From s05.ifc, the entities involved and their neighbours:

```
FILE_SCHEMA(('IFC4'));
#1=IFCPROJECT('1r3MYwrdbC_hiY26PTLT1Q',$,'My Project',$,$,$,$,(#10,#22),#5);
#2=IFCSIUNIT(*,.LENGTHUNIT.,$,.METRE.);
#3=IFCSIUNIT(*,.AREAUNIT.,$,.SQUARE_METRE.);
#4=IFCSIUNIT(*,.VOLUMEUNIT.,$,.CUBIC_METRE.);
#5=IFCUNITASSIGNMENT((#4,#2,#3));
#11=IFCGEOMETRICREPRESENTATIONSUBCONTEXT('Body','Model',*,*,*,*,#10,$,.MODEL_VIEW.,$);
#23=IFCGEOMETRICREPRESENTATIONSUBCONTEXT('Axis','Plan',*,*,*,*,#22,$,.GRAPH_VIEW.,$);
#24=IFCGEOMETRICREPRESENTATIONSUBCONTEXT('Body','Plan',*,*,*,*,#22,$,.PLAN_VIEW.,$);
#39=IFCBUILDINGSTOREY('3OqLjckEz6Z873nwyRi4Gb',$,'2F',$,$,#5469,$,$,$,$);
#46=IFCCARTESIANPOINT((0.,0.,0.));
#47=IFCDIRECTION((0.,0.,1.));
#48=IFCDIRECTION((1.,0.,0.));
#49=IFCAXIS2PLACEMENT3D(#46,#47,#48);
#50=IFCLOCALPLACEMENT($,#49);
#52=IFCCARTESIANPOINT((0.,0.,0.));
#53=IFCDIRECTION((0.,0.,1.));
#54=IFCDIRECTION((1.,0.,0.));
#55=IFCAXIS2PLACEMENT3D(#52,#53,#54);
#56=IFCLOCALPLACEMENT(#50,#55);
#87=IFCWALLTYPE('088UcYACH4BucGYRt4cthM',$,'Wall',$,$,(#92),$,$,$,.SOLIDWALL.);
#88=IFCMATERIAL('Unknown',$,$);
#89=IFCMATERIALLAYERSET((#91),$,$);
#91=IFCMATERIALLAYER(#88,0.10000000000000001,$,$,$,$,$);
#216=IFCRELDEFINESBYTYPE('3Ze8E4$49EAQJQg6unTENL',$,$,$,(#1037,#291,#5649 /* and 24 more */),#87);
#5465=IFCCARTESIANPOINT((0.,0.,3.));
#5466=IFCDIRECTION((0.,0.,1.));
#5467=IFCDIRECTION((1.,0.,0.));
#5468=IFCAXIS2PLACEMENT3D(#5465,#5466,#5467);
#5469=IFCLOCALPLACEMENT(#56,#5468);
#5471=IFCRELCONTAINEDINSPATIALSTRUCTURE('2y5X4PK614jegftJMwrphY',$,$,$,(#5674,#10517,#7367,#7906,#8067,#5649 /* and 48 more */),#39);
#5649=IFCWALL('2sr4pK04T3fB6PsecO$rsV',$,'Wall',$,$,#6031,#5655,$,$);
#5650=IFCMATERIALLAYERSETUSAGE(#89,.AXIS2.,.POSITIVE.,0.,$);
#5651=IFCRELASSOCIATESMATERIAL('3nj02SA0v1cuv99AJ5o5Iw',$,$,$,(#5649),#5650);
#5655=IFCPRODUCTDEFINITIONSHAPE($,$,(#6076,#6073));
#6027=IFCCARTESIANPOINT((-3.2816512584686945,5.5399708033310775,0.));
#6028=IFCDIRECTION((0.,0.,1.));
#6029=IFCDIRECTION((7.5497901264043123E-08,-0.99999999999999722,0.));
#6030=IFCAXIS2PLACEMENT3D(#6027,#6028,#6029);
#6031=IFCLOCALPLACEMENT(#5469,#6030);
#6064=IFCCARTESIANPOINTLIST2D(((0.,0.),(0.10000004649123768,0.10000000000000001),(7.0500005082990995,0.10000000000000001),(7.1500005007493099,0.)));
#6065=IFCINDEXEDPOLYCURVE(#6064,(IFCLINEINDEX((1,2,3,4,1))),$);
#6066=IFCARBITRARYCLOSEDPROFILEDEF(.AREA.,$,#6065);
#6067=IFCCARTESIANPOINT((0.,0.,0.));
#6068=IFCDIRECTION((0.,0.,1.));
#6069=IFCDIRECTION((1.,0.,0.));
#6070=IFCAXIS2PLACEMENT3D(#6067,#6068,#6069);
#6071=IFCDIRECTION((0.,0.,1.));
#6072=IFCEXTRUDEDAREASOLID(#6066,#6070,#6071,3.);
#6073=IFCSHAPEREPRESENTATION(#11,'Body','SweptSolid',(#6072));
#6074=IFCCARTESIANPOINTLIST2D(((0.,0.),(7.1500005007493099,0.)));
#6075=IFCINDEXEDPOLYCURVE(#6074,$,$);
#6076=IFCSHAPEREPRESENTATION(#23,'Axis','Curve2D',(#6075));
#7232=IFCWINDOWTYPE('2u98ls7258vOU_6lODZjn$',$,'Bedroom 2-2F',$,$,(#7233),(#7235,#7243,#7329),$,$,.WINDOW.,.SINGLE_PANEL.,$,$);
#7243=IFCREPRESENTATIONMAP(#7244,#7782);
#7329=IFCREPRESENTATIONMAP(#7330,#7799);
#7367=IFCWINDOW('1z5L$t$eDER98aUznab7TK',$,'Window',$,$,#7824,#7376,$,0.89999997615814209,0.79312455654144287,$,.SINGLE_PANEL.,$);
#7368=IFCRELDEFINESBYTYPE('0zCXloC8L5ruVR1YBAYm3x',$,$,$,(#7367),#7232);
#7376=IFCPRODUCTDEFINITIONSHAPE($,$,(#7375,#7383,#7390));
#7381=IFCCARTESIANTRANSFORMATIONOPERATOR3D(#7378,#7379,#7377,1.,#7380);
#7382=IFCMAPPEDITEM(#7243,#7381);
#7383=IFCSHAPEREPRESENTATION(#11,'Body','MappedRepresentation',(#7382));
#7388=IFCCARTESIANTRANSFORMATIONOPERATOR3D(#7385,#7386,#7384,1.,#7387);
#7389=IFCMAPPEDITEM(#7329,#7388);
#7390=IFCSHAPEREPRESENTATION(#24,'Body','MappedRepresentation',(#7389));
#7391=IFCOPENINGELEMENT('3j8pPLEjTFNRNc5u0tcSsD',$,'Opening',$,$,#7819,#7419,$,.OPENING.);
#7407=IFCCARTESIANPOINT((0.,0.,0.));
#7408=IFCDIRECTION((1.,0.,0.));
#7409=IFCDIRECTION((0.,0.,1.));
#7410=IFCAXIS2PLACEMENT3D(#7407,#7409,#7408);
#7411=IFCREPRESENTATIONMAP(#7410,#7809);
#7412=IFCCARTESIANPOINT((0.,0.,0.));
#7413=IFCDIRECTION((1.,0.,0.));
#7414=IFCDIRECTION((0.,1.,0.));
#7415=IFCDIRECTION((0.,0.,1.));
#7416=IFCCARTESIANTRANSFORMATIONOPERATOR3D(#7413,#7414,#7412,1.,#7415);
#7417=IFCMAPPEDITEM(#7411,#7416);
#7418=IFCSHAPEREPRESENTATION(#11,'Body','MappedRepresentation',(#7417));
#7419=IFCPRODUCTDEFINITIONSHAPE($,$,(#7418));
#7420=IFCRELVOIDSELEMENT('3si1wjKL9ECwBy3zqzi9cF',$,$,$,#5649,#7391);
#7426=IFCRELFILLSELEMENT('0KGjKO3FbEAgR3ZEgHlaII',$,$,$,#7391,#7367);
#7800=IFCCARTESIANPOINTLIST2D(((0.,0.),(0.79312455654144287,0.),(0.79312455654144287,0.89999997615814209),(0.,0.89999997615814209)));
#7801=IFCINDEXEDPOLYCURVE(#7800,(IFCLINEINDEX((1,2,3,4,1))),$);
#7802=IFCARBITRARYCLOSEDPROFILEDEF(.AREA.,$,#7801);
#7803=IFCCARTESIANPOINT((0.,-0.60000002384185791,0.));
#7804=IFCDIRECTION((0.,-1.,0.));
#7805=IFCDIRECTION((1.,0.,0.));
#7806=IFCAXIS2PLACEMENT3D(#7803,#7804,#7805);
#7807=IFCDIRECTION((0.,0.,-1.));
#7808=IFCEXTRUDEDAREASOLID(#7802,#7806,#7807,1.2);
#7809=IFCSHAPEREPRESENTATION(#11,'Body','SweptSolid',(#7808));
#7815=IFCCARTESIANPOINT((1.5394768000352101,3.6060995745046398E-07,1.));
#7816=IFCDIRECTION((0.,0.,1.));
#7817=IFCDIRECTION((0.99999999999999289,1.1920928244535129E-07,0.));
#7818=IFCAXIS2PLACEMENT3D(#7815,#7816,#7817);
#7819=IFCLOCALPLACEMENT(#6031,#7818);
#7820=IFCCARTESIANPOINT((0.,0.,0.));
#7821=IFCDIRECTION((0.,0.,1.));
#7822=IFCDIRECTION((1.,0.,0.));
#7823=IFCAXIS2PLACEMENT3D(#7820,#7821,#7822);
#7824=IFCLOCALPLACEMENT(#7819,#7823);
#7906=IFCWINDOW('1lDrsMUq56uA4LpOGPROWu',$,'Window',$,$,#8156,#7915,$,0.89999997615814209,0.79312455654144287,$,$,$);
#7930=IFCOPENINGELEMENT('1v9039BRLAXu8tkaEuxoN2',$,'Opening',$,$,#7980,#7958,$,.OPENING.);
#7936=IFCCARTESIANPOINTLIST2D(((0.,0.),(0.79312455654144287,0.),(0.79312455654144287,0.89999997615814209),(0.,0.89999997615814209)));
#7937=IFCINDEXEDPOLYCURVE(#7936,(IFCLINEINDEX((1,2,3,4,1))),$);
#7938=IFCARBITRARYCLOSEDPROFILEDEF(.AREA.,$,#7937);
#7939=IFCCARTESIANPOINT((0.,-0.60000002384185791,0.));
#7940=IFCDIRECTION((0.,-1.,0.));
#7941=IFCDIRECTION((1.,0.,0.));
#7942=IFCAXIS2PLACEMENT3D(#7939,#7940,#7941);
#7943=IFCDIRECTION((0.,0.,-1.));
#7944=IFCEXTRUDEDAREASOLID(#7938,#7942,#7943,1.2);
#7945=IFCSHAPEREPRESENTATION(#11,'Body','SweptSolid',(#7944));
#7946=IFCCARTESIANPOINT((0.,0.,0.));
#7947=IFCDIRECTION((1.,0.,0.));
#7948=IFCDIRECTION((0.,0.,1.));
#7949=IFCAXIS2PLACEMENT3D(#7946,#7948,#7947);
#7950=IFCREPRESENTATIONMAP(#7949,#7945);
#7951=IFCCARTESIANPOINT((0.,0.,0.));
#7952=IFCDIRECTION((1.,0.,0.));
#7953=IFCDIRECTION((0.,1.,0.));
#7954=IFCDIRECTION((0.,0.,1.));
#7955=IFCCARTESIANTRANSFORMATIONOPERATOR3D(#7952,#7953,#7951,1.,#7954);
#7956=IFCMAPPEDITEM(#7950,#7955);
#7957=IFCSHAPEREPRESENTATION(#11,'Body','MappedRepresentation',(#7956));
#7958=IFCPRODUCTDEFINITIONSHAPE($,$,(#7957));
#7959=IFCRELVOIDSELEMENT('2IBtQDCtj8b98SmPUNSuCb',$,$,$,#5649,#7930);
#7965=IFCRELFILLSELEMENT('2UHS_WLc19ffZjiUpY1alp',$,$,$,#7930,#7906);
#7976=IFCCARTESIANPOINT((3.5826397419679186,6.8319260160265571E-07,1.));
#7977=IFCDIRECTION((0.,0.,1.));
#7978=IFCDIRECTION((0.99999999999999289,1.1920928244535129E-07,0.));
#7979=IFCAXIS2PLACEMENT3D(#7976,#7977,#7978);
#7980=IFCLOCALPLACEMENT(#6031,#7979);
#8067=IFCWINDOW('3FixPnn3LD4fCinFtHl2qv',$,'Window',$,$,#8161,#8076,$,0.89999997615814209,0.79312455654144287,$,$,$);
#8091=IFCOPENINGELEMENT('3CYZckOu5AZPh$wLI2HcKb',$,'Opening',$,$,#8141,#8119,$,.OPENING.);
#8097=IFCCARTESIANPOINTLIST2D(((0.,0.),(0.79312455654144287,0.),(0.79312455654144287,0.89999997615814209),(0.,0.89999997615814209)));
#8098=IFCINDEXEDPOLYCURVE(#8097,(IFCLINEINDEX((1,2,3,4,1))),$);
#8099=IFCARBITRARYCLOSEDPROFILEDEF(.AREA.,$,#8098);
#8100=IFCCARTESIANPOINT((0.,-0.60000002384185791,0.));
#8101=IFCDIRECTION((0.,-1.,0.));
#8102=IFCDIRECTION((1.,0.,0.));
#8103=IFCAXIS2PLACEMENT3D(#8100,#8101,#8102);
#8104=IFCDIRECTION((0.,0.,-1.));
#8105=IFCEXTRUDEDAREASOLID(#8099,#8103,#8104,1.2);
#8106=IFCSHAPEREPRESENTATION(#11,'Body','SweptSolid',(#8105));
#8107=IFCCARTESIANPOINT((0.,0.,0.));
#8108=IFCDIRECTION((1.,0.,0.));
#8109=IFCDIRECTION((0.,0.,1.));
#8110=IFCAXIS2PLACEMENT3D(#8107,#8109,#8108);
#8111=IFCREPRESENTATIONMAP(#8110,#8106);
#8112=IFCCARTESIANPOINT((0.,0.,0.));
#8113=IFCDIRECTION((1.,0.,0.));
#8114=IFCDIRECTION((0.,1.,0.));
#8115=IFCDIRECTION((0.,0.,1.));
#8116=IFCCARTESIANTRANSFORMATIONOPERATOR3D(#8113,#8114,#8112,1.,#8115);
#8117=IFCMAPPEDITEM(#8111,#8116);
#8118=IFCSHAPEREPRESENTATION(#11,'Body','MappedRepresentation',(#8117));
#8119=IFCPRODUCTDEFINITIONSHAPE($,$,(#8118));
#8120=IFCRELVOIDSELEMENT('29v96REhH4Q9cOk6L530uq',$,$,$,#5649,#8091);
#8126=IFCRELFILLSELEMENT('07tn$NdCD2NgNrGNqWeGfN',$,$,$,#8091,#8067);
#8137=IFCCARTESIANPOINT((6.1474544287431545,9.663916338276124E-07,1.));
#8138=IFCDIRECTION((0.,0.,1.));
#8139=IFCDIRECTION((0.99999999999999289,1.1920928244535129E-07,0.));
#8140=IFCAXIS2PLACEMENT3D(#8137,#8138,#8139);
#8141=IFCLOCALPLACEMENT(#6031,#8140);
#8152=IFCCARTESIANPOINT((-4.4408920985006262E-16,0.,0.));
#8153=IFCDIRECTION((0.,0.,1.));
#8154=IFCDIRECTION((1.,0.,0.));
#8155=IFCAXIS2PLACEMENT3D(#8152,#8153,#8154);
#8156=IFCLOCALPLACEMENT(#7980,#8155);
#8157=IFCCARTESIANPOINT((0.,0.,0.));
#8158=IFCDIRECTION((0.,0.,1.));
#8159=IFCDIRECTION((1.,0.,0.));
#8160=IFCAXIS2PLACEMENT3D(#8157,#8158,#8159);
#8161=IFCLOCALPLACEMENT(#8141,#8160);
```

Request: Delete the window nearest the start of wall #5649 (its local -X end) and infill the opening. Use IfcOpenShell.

```python
import ifcopenshell
import ifcopenshell.api.feature
import ifcopenshell.api.root
import ifcopenshell.geom
import ifcopenshell.util.shape

model = ifcopenshell.open("s05.ifc")
settings = ifcopenshell.geom.settings()


def volume(element):
    """Net volume in cubic metres, openings subtracted."""
    shape = ifcopenshell.geom.create_shape(settings, element)
    return ifcopenshell.util.shape.get_volume(shape.geometry)


window = model.by_guid("1z5L$t$eDER98aUznab7TK")
opening = window.FillsVoids[0].RelatingOpeningElement
wall = opening.VoidsElements[0].RelatingBuildingElement
before = volume(wall)

ifcopenshell.api.root.remove_product(model, product=window)
ifcopenshell.api.feature.remove_feature(model, feature=opening)

after = volume(wall)

print(f"wall volume {before:.3f} -> {after:.3f} m3")

model.write("s05-out.ifc")
```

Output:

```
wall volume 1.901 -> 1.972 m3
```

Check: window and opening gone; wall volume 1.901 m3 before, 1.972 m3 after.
